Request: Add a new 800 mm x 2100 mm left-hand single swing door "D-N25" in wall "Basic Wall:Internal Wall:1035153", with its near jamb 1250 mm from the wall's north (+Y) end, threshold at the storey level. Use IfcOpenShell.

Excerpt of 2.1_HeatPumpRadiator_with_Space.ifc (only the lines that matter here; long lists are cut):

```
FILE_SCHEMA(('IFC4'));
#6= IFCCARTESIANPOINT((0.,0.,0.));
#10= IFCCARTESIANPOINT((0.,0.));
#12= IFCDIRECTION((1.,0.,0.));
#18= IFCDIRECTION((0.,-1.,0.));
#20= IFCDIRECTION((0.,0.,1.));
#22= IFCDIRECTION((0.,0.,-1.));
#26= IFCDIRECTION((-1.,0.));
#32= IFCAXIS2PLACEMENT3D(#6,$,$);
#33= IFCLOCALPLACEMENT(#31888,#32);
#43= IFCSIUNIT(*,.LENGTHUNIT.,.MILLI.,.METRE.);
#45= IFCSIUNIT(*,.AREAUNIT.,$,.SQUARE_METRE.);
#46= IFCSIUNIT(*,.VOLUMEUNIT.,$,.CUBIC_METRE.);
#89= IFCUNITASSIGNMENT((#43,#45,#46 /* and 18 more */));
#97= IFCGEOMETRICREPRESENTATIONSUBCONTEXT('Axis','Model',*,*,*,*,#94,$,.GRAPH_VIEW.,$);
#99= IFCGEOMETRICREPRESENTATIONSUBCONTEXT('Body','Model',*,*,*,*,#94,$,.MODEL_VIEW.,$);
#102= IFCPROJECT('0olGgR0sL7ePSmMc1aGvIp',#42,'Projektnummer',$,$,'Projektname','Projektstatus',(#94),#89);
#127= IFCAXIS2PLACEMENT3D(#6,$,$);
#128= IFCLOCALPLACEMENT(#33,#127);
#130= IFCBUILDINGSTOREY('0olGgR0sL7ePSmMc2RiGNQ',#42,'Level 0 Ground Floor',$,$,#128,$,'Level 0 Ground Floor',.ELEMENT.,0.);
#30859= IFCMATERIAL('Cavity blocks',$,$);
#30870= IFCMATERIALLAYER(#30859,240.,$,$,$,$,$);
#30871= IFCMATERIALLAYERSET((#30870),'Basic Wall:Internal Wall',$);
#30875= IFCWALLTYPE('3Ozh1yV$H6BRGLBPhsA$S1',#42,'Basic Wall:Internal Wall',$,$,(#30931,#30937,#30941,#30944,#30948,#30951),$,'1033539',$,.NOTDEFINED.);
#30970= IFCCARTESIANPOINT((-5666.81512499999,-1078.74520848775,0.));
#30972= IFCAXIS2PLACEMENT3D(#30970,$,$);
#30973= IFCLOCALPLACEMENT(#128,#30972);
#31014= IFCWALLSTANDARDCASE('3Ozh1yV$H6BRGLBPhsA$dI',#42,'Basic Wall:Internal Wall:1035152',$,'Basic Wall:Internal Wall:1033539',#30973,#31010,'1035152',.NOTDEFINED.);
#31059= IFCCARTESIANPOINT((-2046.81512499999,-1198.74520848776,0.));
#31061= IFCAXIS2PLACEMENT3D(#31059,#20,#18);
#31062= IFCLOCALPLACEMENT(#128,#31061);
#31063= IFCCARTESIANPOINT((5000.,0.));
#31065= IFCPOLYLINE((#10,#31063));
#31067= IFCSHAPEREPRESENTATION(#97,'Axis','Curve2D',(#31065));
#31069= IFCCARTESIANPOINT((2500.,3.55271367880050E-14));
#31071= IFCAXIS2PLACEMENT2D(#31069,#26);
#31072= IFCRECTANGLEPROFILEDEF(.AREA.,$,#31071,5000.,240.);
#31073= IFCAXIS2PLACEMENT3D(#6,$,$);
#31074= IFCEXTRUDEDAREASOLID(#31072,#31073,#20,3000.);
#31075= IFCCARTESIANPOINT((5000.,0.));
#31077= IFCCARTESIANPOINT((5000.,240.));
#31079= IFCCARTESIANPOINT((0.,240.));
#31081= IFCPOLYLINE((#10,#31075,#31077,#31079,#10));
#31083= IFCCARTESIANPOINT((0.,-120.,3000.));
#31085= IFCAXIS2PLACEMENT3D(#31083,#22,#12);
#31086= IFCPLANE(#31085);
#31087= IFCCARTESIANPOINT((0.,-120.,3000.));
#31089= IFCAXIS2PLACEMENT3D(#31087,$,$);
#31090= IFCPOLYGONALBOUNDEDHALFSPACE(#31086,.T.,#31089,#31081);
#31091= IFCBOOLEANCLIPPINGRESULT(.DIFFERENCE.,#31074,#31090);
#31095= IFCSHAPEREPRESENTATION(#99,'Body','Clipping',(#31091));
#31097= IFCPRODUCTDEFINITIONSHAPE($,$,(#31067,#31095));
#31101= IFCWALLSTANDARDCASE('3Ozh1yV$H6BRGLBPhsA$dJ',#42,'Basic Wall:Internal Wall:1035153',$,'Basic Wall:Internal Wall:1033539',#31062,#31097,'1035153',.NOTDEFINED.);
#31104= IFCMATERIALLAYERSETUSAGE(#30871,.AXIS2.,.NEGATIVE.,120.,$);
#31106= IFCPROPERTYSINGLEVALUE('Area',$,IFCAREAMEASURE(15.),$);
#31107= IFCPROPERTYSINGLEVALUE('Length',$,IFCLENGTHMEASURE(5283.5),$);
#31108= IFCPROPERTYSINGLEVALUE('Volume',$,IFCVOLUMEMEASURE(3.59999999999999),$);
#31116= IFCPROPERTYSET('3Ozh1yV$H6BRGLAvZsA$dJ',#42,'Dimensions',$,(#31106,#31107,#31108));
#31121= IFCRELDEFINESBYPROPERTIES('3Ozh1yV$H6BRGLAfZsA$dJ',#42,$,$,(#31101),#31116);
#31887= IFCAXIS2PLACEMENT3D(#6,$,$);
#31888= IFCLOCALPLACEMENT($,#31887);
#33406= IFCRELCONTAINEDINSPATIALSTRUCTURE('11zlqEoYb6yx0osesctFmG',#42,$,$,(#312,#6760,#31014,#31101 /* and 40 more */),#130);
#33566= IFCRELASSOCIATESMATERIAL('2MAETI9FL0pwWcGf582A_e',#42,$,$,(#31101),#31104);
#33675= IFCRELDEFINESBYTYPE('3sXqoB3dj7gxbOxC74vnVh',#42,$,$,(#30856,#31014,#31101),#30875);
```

```python
import numpy as np
import ifcopenshell
import ifcopenshell.api.feature
import ifcopenshell.api.geometry
import ifcopenshell.api.pset
import ifcopenshell.api.root
import ifcopenshell.api.spatial
import ifcopenshell.geom
import ifcopenshell.util.element
import ifcopenshell.util.placement
import ifcopenshell.util.representation
import ifcopenshell.util.shape
import ifcopenshell.util.unit

model = ifcopenshell.open("2.1_HeatPumpRadiator_with_Space.ifc")
unit_scale = ifcopenshell.util.unit.calculate_unit_scale(model)
area_scale = ifcopenshell.util.unit.calculate_unit_scale(model, "AREAUNIT")
volume_scale = ifcopenshell.util.unit.calculate_unit_scale(model, "VOLUMEUNIT")
settings = ifcopenshell.geom.settings()


def volume(element):
    """Net volume in cubic metres, openings subtracted."""
    shape = ifcopenshell.geom.create_shape(settings, element)
    return ifcopenshell.util.shape.get_volume(shape.geometry)


wall = model.by_guid("3Ozh1yV$H6BRGLBPhsA$dJ")
storey = ifcopenshell.util.element.get_container(wall, ifc_class="IfcBuildingStorey")
context = ifcopenshell.util.representation.get_context(model, "Model", "Body", "MODEL_VIEW")
before = volume(wall)

width, height, from_end, sill = 0.8, 2.1, 1.25, 0.0  # metres

# The wall runs along its own X axis, and the end named is its -X end.
wall_shape = ifcopenshell.geom.create_shape(settings, wall)
x, y, z = ifcopenshell.util.shape.get_vertices(wall_shape.geometry).T
start = x.min() + from_end
face, thickness = float(y.min()), float(y.max() - y.min())
wall_matrix = ifcopenshell.util.placement.get_local_placement(wall.ObjectPlacement)
level = ifcopenshell.util.placement.get_local_placement(storey.ObjectPlacement)[2, 3]


def in_wall(x, y):
    """Placement at x, y metres in the wall's axes, at sill height."""
    matrix = wall_matrix.copy()
    matrix[:, 3] = wall_matrix @ np.array([x / unit_scale, y / unit_scale, 0.0, 1.0])
    matrix[2, 3] = level + sill / unit_scale
    return matrix


# Opening: a box that overshoots both wall faces by 50 mm.
opening = ifcopenshell.api.root.create_entity(model, ifc_class="IfcOpeningElement", predefined_type="OPENING")
box = ifcopenshell.api.geometry.add_wall_representation(
    model, context=context, length=width, height=height, thickness=thickness + 0.1
)
ifcopenshell.api.geometry.assign_representation(model, product=opening, representation=box)
ifcopenshell.api.geometry.edit_object_placement(model, product=opening, matrix=in_wall(start, face - 0.05), is_si=False)
ifcopenshell.api.feature.add_feature(model, feature=opening, element=wall)

door = ifcopenshell.api.root.create_entity(model, ifc_class="IfcDoor", name="D-N25", predefined_type="DOOR")
door.OverallWidth, door.OverallHeight = width / unit_scale, height / unit_scale
door.OperationType = "SINGLE_SWING_LEFT"
body = ifcopenshell.api.geometry.add_door_representation(
    model,
    context=context,
    overall_width=door.OverallWidth,
    overall_height=door.OverallHeight,
    operation_type="SINGLE_SWING_LEFT",
    lining_properties={"LiningDepth": thickness / unit_scale, "ThresholdDepth": thickness / unit_scale},
)
ifcopenshell.api.geometry.assign_representation(model, product=door, representation=body)
ifcopenshell.api.spatial.assign_container(model, products=[door], relating_structure=storey)
ifcopenshell.api.feature.add_filling(model, opening=opening, element=door)

# The lining spans the wall, so the door starts at the wall face.
ifcopenshell.api.geometry.edit_object_placement(model, product=door, matrix=in_wall(start, face), is_si=False)

after = volume(wall)

# Update the wall's stored quantities.
pset = model.by_id(ifcopenshell.util.element.get_pset(wall, "Dimensions", should_inherit=False)["id"])
ifcopenshell.api.pset.edit_pset(model, pset=pset, properties={
    "Area": model.create_entity("IfcAreaMeasure", after / thickness / area_scale),
    "Volume": model.create_entity("IfcVolumeMeasure", after / volume_scale),
})

print(f"wall volume {before:.3f} -> {after:.3f} m3")

model.write("2.1_HeatPumpRadiator_with_Space_v2.ifc")
```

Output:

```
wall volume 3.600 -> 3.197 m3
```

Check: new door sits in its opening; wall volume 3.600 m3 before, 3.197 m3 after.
